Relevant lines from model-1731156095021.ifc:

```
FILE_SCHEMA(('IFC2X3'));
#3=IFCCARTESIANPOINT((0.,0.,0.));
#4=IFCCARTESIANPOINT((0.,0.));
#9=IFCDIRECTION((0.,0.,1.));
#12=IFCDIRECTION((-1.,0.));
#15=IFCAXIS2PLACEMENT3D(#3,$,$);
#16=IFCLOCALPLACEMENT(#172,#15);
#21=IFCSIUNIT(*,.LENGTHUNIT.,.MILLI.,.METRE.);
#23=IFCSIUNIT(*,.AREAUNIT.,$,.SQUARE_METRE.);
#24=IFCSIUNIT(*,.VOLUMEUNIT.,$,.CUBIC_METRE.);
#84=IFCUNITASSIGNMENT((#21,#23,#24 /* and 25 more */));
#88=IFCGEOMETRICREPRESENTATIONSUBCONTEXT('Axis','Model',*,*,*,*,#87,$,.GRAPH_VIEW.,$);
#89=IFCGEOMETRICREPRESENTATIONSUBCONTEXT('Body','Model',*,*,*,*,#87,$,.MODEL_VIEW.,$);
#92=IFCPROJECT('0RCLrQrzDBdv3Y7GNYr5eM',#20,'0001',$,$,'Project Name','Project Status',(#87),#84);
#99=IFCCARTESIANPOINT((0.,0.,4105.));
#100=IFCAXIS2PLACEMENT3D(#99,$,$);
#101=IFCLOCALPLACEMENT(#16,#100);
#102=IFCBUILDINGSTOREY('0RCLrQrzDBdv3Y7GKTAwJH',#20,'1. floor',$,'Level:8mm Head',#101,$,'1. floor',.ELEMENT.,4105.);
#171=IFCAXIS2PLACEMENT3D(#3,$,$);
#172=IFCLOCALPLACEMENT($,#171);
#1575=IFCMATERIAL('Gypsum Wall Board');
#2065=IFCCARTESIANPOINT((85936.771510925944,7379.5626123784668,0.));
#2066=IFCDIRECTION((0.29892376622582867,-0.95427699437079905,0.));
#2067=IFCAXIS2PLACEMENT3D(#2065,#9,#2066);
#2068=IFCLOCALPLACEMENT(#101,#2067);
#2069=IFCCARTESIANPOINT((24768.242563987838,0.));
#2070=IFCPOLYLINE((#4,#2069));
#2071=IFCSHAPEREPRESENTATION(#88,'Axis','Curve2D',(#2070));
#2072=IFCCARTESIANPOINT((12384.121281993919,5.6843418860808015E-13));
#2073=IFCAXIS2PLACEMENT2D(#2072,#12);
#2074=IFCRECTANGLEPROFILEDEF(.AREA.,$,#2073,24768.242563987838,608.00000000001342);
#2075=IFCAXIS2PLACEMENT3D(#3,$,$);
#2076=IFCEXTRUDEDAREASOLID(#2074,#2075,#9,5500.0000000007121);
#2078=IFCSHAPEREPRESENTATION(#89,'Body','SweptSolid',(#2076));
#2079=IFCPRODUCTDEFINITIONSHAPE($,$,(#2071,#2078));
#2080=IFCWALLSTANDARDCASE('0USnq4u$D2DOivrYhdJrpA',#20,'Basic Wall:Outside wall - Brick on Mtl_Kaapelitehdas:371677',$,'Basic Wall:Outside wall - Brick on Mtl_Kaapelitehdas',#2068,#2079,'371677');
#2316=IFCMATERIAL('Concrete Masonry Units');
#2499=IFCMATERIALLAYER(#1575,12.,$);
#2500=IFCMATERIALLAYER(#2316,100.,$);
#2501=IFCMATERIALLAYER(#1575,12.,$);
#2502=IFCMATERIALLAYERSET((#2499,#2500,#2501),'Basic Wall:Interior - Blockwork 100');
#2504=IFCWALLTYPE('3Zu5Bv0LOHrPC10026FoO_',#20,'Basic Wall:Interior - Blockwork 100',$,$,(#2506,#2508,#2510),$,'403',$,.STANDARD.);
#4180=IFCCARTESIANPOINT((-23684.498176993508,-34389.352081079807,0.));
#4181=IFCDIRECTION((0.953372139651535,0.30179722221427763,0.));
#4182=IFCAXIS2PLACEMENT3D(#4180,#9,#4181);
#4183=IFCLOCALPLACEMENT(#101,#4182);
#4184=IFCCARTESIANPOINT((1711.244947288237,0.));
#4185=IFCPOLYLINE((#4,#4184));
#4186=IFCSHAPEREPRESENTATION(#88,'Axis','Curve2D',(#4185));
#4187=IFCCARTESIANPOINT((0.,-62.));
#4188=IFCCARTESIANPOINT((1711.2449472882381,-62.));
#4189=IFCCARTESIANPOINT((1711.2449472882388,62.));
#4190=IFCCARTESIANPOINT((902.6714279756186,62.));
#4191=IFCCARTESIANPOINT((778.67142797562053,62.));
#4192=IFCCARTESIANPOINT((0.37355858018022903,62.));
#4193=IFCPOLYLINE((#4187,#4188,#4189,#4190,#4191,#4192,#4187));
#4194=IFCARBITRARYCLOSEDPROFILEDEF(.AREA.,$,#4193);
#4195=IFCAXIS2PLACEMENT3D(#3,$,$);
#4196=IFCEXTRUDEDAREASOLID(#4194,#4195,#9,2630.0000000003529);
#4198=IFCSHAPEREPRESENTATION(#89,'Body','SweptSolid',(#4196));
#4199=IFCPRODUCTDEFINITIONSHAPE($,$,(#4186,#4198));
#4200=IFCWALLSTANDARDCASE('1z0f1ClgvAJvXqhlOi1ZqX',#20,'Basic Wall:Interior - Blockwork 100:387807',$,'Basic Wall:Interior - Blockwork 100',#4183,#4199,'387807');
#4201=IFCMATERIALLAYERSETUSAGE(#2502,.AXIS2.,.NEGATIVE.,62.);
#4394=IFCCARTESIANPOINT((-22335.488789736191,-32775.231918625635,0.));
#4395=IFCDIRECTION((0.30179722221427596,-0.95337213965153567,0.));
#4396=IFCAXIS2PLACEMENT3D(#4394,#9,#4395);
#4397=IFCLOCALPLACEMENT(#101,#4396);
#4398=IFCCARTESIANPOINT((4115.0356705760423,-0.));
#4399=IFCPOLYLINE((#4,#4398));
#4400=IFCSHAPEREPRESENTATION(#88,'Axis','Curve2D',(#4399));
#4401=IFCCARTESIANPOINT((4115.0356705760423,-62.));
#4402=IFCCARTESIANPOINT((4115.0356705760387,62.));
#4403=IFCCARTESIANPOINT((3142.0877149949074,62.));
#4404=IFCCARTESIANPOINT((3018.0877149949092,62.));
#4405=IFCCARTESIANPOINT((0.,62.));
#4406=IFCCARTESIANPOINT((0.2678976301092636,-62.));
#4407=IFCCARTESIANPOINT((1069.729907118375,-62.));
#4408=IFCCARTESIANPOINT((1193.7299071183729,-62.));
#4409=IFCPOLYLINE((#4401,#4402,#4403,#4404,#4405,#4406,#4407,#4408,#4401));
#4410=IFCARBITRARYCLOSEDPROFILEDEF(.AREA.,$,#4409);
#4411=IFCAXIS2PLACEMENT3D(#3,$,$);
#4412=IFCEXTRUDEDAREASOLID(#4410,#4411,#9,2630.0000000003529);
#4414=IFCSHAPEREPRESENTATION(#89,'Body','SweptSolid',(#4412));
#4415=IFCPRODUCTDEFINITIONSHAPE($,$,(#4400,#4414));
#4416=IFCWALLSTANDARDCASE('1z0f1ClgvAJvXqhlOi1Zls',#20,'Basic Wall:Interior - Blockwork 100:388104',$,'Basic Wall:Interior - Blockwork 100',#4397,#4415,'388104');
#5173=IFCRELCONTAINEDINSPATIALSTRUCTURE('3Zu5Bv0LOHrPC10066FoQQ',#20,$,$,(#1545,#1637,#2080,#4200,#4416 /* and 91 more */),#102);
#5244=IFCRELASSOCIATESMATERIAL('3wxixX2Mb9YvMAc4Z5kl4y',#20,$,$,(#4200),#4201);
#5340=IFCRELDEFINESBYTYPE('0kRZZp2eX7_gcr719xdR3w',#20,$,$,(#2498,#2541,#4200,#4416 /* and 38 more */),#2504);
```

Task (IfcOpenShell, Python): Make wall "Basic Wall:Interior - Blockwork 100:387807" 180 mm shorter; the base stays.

```python
import ifcopenshell
import ifcopenshell.geom
import ifcopenshell.util.representation
import ifcopenshell.util.shape

model = ifcopenshell.open("model-1731156095021.ifc")
settings = ifcopenshell.geom.settings()


def volume(element):
    """Net volume in cubic metres, openings subtracted."""
    shape = ifcopenshell.geom.create_shape(settings, element)
    return ifcopenshell.util.shape.get_volume(shape.geometry)


wall = model.by_id(4200)
before = volume(wall)

body = ifcopenshell.util.representation.get_representation(wall, "Model", "Body")
solid = body.Items[0]
old_height = solid.Depth
solid.Depth -= 180.0
after = volume(wall)

print(f"height {old_height:g} -> {solid.Depth:g}, volume {before:.3f} -> {after:.3f} m3")

model.write("model-1731156095021-out.ifc")
```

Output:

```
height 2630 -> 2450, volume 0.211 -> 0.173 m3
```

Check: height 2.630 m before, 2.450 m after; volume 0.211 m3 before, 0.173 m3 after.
